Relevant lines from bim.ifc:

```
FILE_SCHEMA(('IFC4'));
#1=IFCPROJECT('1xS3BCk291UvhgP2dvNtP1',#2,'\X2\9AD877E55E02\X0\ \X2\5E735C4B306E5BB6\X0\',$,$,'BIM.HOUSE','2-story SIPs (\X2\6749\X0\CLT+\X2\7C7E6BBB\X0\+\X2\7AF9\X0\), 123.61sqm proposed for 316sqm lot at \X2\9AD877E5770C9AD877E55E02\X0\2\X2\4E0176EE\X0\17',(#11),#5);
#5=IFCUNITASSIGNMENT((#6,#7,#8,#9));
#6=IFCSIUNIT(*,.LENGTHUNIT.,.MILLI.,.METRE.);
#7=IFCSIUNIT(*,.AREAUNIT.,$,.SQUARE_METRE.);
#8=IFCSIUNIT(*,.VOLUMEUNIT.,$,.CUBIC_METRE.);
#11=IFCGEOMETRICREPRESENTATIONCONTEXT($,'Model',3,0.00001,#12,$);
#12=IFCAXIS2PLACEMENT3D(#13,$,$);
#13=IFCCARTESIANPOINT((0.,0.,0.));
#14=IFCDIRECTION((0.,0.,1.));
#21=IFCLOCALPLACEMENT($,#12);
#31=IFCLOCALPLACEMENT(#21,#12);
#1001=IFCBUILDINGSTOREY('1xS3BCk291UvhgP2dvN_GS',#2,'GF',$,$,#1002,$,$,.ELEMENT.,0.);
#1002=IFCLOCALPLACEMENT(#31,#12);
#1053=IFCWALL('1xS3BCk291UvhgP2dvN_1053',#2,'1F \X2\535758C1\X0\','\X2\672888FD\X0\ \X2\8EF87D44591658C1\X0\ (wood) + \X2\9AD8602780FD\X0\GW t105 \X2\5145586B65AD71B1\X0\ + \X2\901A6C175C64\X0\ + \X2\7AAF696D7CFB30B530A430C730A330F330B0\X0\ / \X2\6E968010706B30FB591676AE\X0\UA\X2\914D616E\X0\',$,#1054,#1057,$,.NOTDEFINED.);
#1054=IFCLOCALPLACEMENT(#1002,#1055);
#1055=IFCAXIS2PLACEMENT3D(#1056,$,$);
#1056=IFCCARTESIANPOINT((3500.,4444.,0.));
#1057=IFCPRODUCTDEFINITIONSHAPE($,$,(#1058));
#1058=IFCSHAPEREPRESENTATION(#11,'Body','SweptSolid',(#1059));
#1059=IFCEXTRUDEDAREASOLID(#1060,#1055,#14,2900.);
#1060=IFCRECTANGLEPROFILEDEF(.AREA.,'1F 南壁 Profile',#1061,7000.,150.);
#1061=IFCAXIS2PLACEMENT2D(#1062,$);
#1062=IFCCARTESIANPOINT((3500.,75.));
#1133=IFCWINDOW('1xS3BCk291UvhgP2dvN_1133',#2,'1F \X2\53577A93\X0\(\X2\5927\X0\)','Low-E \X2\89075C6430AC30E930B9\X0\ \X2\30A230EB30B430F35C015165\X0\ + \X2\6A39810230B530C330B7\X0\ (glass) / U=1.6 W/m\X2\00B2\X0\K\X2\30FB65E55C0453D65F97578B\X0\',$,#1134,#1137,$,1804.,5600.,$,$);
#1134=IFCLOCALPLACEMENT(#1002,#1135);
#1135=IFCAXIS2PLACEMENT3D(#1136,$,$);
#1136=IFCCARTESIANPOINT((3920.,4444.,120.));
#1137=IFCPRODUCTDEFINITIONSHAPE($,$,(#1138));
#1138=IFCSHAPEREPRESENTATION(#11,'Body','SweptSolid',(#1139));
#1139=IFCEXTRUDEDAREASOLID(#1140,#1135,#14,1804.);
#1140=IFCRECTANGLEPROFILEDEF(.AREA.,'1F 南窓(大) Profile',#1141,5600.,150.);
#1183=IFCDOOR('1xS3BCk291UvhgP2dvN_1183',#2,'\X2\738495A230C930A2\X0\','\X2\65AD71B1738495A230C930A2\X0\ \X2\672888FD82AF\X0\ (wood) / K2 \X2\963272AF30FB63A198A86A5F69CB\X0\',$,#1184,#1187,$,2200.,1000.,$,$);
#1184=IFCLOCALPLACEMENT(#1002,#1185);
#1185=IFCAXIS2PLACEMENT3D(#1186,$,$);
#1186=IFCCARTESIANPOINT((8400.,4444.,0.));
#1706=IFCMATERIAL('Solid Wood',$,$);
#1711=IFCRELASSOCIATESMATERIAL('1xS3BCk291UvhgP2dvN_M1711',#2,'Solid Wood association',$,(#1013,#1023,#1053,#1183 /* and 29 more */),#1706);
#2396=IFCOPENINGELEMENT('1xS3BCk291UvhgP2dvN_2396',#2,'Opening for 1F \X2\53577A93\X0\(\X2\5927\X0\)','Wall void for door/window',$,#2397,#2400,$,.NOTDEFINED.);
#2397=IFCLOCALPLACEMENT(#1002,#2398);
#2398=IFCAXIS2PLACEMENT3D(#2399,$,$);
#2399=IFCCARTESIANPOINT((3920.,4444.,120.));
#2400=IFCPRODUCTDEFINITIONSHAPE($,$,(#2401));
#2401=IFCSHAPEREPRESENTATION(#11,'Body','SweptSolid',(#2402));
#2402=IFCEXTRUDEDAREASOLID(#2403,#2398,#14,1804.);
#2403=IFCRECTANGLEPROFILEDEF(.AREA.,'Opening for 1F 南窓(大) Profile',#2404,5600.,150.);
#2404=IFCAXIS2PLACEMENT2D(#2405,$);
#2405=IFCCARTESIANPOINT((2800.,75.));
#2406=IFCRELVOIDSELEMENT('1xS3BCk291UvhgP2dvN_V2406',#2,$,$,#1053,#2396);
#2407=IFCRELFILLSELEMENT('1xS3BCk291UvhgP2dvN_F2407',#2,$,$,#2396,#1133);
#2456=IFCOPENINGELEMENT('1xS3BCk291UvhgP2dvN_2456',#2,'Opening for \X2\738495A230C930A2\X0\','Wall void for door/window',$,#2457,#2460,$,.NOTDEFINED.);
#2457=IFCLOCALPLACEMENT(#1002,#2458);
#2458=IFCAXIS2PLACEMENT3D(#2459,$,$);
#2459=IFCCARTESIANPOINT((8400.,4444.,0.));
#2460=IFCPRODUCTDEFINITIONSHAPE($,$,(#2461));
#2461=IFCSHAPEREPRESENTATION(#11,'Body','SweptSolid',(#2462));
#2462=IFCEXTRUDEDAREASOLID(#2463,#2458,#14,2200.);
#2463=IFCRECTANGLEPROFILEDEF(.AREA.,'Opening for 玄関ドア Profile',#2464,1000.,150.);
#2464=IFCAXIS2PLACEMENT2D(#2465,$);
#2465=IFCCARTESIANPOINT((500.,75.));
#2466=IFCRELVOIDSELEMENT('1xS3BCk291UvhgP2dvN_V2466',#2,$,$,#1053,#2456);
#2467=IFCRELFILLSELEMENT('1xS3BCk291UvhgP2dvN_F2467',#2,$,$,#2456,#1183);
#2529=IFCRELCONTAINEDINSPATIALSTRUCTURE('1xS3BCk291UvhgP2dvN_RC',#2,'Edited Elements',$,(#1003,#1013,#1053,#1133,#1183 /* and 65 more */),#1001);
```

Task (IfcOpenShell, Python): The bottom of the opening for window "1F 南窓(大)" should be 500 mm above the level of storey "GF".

```python
import numpy as np
import ifcopenshell
import ifcopenshell.api.geometry
import ifcopenshell.geom
import ifcopenshell.util.element
import ifcopenshell.util.placement
import ifcopenshell.util.shape
import ifcopenshell.util.unit

model = ifcopenshell.open("bim.ifc")
unit_scale = ifcopenshell.util.unit.calculate_unit_scale(model)

window = model.by_guid("1xS3BCk291UvhgP2dvN_1133")
opening = window.FillsVoids[0].RelatingOpeningElement
storey = ifcopenshell.util.element.get_container(window, ifc_class="IfcBuildingStorey")
level = ifcopenshell.util.placement.get_local_placement(storey.ObjectPlacement)[2, 3]

# The opening's origin need not be at the sill, so measure its lowest point.
shape = ifcopenshell.geom.create_shape(ifcopenshell.geom.settings(), opening)
bottom = ifcopenshell.util.shape.get_shape_bottom_elevation(shape, shape.geometry) / unit_scale
dz = level + 0.5 / unit_scale - bottom

shift = np.array([0.0, 0.0, dz])
# The window is not placed relative to its opening, so move both.
for product in (opening, window):
    matrix = ifcopenshell.util.placement.get_local_placement(product.ObjectPlacement)
    matrix[:3, 3] += shift
    ifcopenshell.api.geometry.edit_object_placement(model, product=product, matrix=matrix, is_si=False)

print(f"moved by {dz * unit_scale:+.3f} m")

model.write("bim_rev.ifc")
```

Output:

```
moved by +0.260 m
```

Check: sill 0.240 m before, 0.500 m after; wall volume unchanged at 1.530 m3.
